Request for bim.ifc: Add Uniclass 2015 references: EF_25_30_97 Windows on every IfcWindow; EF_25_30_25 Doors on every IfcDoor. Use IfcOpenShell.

First a look at what the model holds.

```python
import ifcopenshell

model = ifcopenshell.open("bim.ifc")
print(model.schema)
print("classifications:", [c.Name for c in model.by_type("IfcClassification")])
for ifc_class in ("IfcDoor", "IfcRoof", "IfcStair", "IfcWall", "IfcWindow"):
    print(ifc_class, len(model.by_type(ifc_class)))
```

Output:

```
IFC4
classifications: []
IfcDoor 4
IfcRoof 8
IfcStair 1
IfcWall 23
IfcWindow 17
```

```python
import ifcopenshell
import ifcopenshell.api.classification

model = ifcopenshell.open("bim.ifc")

system = ifcopenshell.api.classification.add_classification(model, classification="Uniclass 2015")

codes = {
    "IfcWindow": ("EF_25_30_97", "Windows"),
    "IfcDoor": ("EF_25_30_25", "Doors"),
}
for ifc_class, (code, name) in codes.items():
    products = model.by_type(ifc_class)
    ifcopenshell.api.classification.add_reference(
        model, products=products, classification=system, identification=code, name=name
    )
    print(code, len(products))

model.write("bim_edited.ifc")
```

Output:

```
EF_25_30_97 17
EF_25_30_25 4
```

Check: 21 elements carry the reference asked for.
